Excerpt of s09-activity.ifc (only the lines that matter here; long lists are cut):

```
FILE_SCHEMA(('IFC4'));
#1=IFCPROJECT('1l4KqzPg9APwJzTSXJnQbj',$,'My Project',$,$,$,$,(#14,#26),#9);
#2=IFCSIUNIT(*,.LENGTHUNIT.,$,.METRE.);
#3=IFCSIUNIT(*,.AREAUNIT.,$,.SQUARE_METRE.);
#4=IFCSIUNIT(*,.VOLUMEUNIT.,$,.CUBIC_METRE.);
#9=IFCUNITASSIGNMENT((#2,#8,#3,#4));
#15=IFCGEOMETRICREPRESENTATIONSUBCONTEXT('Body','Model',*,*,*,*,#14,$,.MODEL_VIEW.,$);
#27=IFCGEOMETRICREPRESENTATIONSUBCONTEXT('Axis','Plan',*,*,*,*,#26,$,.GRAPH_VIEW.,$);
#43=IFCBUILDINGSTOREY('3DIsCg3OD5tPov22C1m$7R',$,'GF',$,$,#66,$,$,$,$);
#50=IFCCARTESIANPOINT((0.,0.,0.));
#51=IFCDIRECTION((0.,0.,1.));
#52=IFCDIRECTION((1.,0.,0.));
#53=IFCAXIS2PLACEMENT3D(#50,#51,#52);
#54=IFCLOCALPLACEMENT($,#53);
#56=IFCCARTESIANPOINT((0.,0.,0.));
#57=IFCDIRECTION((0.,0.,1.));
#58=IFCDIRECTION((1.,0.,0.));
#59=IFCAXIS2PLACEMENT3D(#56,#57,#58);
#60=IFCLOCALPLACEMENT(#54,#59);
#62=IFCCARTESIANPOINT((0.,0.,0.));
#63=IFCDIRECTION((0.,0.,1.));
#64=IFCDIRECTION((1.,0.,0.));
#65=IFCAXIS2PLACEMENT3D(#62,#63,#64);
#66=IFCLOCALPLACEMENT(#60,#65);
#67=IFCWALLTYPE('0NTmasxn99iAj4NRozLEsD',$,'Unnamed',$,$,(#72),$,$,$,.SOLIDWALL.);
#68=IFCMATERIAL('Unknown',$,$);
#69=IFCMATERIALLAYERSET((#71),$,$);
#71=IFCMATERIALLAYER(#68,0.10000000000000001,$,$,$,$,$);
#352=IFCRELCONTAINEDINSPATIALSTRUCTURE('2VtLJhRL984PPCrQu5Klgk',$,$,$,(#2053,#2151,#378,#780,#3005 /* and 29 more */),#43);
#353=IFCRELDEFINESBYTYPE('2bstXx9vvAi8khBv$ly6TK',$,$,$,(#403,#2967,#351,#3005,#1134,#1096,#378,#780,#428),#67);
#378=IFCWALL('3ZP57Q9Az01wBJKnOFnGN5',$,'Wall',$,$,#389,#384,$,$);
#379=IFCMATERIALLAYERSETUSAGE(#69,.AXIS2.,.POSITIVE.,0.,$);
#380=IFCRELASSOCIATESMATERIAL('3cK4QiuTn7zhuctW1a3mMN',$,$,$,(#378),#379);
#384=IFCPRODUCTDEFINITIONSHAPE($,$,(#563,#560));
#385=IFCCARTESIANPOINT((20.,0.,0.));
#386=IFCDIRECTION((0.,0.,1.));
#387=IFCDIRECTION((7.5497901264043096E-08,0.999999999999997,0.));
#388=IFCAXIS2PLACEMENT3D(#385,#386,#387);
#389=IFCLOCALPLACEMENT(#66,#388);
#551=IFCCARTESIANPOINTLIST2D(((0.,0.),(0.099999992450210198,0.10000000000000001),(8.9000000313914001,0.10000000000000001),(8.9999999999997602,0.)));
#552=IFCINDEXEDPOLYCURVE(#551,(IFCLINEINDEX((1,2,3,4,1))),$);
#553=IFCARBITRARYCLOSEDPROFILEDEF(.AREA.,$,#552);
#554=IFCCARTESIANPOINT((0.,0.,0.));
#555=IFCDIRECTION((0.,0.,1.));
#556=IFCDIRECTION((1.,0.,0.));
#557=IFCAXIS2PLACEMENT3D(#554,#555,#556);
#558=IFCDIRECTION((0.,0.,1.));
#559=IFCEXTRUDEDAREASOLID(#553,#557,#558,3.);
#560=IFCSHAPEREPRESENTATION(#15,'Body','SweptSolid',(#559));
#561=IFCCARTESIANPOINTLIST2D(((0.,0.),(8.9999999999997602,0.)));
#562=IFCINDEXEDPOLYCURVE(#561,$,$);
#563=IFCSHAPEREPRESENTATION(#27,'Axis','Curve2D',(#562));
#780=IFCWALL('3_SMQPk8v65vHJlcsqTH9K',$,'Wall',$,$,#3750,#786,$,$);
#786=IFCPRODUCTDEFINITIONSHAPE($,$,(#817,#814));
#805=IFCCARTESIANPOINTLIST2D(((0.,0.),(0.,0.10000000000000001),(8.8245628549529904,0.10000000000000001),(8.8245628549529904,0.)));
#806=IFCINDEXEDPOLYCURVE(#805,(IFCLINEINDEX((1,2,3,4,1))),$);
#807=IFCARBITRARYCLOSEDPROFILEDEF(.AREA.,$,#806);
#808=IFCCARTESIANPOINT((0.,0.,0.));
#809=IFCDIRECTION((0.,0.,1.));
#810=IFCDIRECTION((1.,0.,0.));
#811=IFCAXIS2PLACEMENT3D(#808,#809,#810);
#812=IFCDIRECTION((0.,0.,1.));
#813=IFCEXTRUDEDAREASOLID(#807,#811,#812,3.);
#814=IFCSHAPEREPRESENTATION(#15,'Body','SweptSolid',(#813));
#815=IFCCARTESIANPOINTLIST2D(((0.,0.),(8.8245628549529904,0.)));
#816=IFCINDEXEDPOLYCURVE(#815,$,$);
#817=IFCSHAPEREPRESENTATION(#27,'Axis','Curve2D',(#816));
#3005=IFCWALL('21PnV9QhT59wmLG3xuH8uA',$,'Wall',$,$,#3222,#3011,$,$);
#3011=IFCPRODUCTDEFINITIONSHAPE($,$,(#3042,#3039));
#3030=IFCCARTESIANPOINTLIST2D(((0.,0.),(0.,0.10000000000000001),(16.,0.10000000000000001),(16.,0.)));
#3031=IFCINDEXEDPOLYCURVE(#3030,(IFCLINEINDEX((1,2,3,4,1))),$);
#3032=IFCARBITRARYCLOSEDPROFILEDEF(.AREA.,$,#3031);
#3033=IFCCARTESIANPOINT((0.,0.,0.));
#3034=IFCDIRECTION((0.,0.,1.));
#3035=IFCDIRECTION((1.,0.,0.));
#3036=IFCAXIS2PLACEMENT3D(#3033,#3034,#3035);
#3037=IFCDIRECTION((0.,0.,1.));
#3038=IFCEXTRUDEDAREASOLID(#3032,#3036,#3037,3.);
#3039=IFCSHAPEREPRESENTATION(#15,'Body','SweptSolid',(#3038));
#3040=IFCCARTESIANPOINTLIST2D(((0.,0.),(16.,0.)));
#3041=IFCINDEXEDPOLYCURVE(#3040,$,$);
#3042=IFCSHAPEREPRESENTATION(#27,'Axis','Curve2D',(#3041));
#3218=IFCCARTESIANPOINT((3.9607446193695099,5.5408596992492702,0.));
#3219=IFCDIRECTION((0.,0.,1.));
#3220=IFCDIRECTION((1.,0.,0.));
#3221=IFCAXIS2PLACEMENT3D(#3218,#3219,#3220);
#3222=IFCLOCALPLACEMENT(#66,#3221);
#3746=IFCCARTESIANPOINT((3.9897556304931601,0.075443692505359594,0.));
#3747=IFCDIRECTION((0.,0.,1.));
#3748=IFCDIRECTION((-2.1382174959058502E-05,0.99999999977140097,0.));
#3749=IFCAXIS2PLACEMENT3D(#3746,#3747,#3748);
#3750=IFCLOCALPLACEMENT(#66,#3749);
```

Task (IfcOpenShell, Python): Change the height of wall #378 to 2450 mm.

```python
import ifcopenshell
import ifcopenshell.geom
import ifcopenshell.util.representation
import ifcopenshell.util.shape
import ifcopenshell.util.unit

model = ifcopenshell.open("s09-activity.ifc")
unit_scale = ifcopenshell.util.unit.calculate_unit_scale(model)
settings = ifcopenshell.geom.settings()


def volume(element):
    """Net volume in cubic metres, openings subtracted."""
    shape = ifcopenshell.geom.create_shape(settings, element)
    return ifcopenshell.util.shape.get_volume(shape.geometry)


wall = model.by_id(378)
before = volume(wall)

body = ifcopenshell.util.representation.get_representation(wall, "Model", "Body")
solid = body.Items[0]
old_height = solid.Depth
solid.Depth = 2.45 / unit_scale
after = volume(wall)

print(f"height {old_height:g} -> {solid.Depth:g}, volume {before:.3f} -> {after:.3f} m3")

model.write("s09-activity_rev.ifc")
```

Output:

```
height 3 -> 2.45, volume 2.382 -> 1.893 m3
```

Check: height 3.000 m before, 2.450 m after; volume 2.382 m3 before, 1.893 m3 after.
